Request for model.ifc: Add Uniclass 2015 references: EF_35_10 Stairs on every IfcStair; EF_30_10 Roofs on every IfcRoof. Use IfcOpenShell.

First a look at what the model holds.

```python
import ifcopenshell

model = ifcopenshell.open("model.ifc")
print(model.schema)
print("classifications:", [c.Name for c in model.by_type("IfcClassification")])
for ifc_class in ("IfcDoor", "IfcRoof", "IfcStair", "IfcWall", "IfcWindow"):
    print(ifc_class, len(model.by_type(ifc_class)))
```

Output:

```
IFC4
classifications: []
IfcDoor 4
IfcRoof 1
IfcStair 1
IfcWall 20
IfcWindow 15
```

```python
import ifcopenshell
import ifcopenshell.api.classification

model = ifcopenshell.open("model.ifc")

system = ifcopenshell.api.classification.add_classification(model, classification="Uniclass 2015")

codes = {
    "IfcStair": ("EF_35_10", "Stairs"),
    "IfcRoof": ("EF_30_10", "Roofs"),
}
for ifc_class, (code, name) in codes.items():
    products = model.by_type(ifc_class)
    ifcopenshell.api.classification.add_reference(
        model, products=products, classification=system, identification=code, name=name
    )
    print(code, len(products))

model.write("model-out.ifc")
```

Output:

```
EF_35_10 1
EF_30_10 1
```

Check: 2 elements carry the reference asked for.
